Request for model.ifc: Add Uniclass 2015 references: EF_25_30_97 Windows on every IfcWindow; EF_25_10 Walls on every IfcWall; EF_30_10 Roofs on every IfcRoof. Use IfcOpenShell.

First a look at what the model holds.

```python
import ifcopenshell

model = ifcopenshell.open("model.ifc")
print(model.schema)
print("classifications:", [c.Name for c in model.by_type("IfcClassification")])
for ifc_class in ("IfcDoor", "IfcRoof", "IfcStair", "IfcWall", "IfcWindow"):
    print(ifc_class, len(model.by_type(ifc_class)))
```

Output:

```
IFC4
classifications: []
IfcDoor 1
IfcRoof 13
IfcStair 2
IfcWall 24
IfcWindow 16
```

```python
import ifcopenshell
import ifcopenshell.api.classification

model = ifcopenshell.open("model.ifc")

system = ifcopenshell.api.classification.add_classification(model, classification="Uniclass 2015")

codes = {
    "IfcWindow": ("EF_25_30_97", "Windows"),
    "IfcWall": ("EF_25_10", "Walls"),
    "IfcRoof": ("EF_30_10", "Roofs"),
}
for ifc_class, (code, name) in codes.items():
    products = model.by_type(ifc_class)
    ifcopenshell.api.classification.add_reference(
        model, products=products, classification=system, identification=code, name=name
    )
    print(code, len(products))

model.write("model_v2.ifc")
```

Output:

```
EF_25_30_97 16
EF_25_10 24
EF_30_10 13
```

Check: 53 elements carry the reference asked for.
